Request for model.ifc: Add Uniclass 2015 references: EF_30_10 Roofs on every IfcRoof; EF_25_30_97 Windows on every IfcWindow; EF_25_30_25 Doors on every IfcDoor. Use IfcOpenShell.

First a look at what the model holds.

```python
import ifcopenshell

model = ifcopenshell.open("model.ifc")
print(model.schema)
print("classifications:", [c.Name for c in model.by_type("IfcClassification")])
for ifc_class in ("IfcDoor", "IfcRoof", "IfcStair", "IfcWall", "IfcWindow"):
    print(ifc_class, len(model.by_type(ifc_class)))
```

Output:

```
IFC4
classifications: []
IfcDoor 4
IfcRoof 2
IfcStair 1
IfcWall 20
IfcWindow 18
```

```python
import ifcopenshell
import ifcopenshell.api.classification

model = ifcopenshell.open("model.ifc")

system = ifcopenshell.api.classification.add_classification(model, classification="Uniclass 2015")

codes = {
    "IfcRoof": ("EF_30_10", "Roofs"),
    "IfcWindow": ("EF_25_30_97", "Windows"),
    "IfcDoor": ("EF_25_30_25", "Doors"),
}
for ifc_class, (code, name) in codes.items():
    products = model.by_type(ifc_class)
    ifcopenshell.api.classification.add_reference(
        model, products=products, classification=system, identification=code, name=name
    )
    print(code, len(products))

model.write("model-out.ifc")
```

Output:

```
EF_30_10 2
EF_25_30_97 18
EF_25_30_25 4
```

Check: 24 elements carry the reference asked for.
